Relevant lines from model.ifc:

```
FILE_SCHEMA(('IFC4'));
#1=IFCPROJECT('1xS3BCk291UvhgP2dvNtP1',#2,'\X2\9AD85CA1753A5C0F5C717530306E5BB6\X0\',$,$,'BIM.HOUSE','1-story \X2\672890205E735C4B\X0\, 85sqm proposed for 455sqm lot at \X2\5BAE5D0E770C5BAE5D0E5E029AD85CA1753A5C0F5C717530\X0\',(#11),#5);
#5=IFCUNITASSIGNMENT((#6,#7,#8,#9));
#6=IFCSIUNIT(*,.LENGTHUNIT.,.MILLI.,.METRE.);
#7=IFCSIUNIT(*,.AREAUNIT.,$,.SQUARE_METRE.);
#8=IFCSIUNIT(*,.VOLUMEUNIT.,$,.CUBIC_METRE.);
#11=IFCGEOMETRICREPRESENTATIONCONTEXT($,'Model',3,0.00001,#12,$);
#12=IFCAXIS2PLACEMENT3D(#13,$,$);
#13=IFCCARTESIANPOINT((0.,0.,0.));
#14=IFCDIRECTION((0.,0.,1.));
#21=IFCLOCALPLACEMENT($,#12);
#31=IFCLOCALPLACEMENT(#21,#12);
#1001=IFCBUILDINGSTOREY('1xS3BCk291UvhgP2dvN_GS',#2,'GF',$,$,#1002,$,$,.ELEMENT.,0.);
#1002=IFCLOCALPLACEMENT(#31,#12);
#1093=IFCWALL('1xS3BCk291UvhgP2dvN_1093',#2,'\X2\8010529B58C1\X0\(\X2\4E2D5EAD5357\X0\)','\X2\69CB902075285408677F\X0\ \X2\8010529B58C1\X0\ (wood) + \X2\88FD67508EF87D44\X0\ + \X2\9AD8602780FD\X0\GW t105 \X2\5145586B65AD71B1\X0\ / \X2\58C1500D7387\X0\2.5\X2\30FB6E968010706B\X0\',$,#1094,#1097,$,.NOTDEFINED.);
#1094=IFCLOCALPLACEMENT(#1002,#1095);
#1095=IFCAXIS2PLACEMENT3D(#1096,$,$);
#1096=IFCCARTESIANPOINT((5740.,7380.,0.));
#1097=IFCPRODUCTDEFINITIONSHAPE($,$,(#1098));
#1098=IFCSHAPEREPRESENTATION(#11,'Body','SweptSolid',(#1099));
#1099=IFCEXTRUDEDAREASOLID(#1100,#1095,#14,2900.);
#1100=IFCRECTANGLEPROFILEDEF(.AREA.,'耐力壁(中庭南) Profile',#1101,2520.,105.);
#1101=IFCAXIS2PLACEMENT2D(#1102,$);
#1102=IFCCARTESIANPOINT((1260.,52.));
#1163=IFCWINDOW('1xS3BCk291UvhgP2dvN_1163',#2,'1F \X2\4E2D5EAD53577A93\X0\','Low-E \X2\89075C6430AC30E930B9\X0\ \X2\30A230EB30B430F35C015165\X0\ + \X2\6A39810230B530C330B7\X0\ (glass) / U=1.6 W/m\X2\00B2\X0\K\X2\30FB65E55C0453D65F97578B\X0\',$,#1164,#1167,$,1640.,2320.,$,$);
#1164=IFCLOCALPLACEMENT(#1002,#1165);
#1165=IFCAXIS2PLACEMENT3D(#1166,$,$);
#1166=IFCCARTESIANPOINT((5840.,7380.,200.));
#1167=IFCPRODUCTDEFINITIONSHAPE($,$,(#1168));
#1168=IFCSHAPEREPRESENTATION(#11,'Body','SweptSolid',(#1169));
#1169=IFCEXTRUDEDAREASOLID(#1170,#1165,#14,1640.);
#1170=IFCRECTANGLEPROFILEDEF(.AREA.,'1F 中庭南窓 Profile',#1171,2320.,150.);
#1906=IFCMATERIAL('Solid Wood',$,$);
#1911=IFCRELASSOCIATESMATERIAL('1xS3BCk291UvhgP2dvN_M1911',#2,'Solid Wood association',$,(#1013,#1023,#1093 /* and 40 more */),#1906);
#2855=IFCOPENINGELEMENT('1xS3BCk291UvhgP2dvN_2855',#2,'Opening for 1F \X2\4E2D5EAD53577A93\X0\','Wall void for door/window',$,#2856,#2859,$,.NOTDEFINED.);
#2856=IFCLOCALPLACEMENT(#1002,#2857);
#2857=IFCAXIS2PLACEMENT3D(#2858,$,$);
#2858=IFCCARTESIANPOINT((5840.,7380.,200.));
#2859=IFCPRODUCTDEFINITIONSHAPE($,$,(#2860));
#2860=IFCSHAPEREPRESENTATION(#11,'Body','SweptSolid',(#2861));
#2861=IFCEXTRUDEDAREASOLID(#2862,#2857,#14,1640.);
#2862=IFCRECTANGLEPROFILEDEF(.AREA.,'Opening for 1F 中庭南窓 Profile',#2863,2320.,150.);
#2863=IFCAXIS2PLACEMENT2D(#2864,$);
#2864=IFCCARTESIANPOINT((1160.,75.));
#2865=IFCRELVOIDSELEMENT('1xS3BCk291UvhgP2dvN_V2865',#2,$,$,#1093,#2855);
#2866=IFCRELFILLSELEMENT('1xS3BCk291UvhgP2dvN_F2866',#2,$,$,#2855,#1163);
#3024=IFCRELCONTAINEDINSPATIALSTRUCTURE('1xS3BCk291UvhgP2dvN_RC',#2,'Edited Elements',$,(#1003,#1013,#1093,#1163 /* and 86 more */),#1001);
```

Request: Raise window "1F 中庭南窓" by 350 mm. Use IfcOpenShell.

```python
import numpy as np
import ifcopenshell
import ifcopenshell.api.geometry
import ifcopenshell.util.placement
import ifcopenshell.util.unit

model = ifcopenshell.open("model.ifc")
unit_scale = ifcopenshell.util.unit.calculate_unit_scale(model)

window = model.by_id(1163)
opening = window.FillsVoids[0].RelatingOpeningElement
dz = 0.35 / unit_scale

shift = np.array([0.0, 0.0, dz])
# The window is not placed relative to its opening, so move both.
for product in (opening, window):
    matrix = ifcopenshell.util.placement.get_local_placement(product.ObjectPlacement)
    matrix[:3, 3] += shift
    ifcopenshell.api.geometry.edit_object_placement(model, product=product, matrix=matrix, is_si=False)

print(f"moved by {dz * unit_scale:+.3f} m")

model.write("model_edited.ifc")
```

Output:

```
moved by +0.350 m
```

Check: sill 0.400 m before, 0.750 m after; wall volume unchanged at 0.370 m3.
